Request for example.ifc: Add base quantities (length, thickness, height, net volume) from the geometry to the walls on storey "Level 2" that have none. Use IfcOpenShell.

First a look at what the model holds.

```python
import ifcopenshell
import ifcopenshell.util.element
import ifcopenshell.util.unit

model = ifcopenshell.open("example.ifc")
print(model.schema)
for unit_type in ("LENGTHUNIT", "AREAUNIT", "VOLUMEUNIT"):
    print(unit_type, ifcopenshell.util.unit.calculate_unit_scale(model, unit_type))
storey = next(s for s in model.by_type("IfcBuildingStorey") if s.Name == "Level 2")
walls = [e for e in ifcopenshell.util.element.get_decomposition(storey) if e.is_a("IfcWall")]
for e in sorted(walls, key=lambda e: e.id()):
    print(e.id(), e.is_a(), e.Name, list(ifcopenshell.util.element.get_psets(e, qtos_only=True)), sep=" | ")
```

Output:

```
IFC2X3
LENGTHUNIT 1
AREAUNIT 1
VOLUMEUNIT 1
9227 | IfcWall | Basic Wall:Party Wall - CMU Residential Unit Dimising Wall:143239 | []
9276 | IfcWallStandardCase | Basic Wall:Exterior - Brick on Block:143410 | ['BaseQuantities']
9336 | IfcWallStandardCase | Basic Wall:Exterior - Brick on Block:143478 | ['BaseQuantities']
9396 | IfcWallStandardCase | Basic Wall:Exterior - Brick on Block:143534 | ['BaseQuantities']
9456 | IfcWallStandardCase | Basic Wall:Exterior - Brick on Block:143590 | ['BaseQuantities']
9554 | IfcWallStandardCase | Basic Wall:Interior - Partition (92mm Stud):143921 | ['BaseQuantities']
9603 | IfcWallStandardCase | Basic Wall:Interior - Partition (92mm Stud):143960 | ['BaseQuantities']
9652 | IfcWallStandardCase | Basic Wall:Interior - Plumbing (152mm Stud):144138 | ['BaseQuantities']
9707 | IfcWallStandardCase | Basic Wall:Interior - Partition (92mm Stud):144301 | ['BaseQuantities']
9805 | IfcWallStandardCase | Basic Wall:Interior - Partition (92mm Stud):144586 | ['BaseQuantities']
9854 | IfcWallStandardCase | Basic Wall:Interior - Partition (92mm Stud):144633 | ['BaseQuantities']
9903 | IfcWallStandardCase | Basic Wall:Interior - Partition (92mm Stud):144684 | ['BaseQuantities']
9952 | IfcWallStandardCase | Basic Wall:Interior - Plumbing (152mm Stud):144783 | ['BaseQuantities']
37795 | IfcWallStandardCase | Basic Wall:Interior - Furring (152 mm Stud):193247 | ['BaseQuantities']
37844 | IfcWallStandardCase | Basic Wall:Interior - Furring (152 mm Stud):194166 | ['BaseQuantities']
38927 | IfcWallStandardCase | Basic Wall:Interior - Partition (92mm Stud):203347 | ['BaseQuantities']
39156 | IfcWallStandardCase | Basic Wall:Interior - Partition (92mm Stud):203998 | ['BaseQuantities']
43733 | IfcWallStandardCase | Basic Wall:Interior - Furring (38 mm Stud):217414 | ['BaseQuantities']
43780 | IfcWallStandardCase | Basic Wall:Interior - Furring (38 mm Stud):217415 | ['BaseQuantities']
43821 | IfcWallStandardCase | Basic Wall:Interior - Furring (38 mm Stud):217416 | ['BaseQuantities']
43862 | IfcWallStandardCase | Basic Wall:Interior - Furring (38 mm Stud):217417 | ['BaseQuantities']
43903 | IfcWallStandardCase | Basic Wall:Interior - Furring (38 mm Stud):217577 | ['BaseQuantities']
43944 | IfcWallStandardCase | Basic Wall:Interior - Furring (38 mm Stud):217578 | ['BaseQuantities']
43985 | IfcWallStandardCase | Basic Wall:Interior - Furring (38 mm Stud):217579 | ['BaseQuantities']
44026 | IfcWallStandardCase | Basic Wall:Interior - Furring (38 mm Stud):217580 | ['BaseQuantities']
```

```python
import ifcopenshell
import ifcopenshell.api.pset
import ifcopenshell.geom
import ifcopenshell.util.element
import ifcopenshell.util.shape
import ifcopenshell.util.unit

model = ifcopenshell.open("example.ifc")
unit_scale = ifcopenshell.util.unit.calculate_unit_scale(model)
volume_scale = ifcopenshell.util.unit.calculate_unit_scale(model, "VOLUMEUNIT")
settings = ifcopenshell.geom.settings()

storey = next(s for s in model.by_type("IfcBuildingStorey") if s.Name == "Level 2")
walls = [e for e in ifcopenshell.util.element.get_decomposition(storey) if e.is_a("IfcWall")]

for e in sorted(walls, key=lambda e: e.id()):
    if ifcopenshell.util.element.get_psets(e, qtos_only=True, should_inherit=False):
        continue
    # Geometry comes back in metres, in the element's own axes.
    shape = ifcopenshell.geom.create_shape(settings, e)
    values = {
        "Length": ifcopenshell.util.shape.get_x(shape.geometry) / unit_scale,
        "Width": ifcopenshell.util.shape.get_y(shape.geometry) / unit_scale,
        "Height": ifcopenshell.util.shape.get_z(shape.geometry) / unit_scale,
        "NetVolume": ifcopenshell.util.shape.get_volume(shape.geometry) / volume_scale,
    }
    qto = ifcopenshell.api.pset.add_qto(model, product=e, name="BaseQuantities")
    ifcopenshell.api.pset.edit_qto(model, qto=qto, properties=values)
    print(e.id(), {k: round(v, 3) for k, v in values.items()})

model.write("example_edited.ifc")
```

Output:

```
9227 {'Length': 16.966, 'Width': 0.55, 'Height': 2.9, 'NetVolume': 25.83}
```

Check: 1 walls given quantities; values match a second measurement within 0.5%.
